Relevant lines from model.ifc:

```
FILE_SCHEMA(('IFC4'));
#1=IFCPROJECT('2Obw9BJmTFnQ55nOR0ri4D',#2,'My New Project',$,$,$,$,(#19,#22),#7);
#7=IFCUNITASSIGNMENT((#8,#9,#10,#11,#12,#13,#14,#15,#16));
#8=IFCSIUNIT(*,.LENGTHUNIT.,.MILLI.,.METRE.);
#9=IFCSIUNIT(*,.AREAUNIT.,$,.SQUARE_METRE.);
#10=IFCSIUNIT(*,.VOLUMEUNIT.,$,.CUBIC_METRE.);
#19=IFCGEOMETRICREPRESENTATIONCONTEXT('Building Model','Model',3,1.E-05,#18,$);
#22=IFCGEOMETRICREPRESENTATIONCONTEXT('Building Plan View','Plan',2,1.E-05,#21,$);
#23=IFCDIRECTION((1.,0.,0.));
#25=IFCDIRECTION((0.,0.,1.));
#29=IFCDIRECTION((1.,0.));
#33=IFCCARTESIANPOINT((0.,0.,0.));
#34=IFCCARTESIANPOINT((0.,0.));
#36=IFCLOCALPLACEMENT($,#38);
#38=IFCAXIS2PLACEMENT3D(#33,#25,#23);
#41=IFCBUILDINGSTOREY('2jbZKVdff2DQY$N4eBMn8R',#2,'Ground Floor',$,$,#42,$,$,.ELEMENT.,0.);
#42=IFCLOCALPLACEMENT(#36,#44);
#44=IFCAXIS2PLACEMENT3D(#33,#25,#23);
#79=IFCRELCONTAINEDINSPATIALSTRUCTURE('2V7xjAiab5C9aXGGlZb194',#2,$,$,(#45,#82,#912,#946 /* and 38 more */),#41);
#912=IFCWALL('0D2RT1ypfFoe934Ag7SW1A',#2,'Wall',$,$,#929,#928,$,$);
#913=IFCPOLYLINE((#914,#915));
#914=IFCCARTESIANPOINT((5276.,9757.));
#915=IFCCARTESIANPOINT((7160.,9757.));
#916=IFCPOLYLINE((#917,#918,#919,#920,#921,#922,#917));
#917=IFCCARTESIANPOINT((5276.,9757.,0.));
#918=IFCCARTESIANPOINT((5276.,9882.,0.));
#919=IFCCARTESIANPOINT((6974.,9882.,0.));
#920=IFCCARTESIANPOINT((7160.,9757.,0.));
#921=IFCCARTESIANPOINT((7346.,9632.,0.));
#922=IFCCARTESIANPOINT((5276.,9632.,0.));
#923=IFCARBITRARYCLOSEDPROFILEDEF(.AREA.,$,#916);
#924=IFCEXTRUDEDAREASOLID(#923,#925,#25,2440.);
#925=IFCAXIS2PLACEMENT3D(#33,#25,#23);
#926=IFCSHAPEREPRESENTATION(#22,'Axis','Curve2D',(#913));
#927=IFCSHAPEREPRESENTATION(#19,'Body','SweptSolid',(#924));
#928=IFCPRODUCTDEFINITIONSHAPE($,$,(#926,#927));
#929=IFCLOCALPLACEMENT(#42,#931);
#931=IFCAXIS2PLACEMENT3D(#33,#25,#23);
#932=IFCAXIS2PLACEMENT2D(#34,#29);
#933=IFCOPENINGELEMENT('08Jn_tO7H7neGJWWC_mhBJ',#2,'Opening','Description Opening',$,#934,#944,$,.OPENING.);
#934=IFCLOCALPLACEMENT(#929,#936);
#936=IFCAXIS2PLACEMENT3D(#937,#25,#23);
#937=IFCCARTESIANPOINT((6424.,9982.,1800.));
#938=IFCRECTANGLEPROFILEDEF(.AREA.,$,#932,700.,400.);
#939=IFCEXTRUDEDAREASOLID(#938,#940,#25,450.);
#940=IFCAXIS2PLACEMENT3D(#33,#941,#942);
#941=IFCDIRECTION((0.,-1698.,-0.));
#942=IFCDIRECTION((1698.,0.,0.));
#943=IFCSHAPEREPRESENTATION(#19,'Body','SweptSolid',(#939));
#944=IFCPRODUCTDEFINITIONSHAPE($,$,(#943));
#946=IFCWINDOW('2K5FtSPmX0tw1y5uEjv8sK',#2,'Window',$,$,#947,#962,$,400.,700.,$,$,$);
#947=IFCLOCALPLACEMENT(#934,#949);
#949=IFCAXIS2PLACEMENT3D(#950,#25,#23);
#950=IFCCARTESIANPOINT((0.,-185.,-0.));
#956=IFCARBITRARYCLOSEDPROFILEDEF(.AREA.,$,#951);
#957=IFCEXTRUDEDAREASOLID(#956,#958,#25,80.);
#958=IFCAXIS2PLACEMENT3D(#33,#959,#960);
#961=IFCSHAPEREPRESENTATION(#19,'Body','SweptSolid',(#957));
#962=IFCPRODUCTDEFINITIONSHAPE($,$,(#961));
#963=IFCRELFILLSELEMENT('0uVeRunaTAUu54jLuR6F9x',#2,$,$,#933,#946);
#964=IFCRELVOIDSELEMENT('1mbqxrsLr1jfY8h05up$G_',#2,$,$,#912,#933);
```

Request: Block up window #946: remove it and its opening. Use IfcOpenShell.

```python
import ifcopenshell
import ifcopenshell.api.feature
import ifcopenshell.api.root
import ifcopenshell.geom
import ifcopenshell.util.shape

model = ifcopenshell.open("model.ifc")
settings = ifcopenshell.geom.settings()


def volume(element):
    """Net volume in cubic metres, openings subtracted."""
    shape = ifcopenshell.geom.create_shape(settings, element)
    return ifcopenshell.util.shape.get_volume(shape.geometry)


window = model.by_guid("2K5FtSPmX0tw1y5uEjv8sK")
opening = window.FillsVoids[0].RelatingOpeningElement
wall = opening.VoidsElements[0].RelatingBuildingElement
before = volume(wall)

ifcopenshell.api.root.remove_product(model, product=window)
ifcopenshell.api.feature.remove_feature(model, feature=opening)

after = volume(wall)

print(f"wall volume {before:.3f} -> {after:.3f} m3")

model.write("model_rev.ifc")
```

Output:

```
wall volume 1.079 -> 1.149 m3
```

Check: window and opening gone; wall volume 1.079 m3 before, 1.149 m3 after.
